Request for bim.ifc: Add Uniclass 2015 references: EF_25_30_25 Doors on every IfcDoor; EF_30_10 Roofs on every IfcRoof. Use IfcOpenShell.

First a look at what the model holds.

```python
import ifcopenshell

model = ifcopenshell.open("bim.ifc")
print(model.schema)
print("classifications:", [c.Name for c in model.by_type("IfcClassification")])
for ifc_class in ("IfcDoor", "IfcRoof", "IfcStair", "IfcWall", "IfcWindow"):
    print(ifc_class, len(model.by_type(ifc_class)))
```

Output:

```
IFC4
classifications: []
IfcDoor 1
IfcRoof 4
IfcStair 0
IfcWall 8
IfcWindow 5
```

```python
import ifcopenshell
import ifcopenshell.api.classification

model = ifcopenshell.open("bim.ifc")

system = ifcopenshell.api.classification.add_classification(model, classification="Uniclass 2015")

codes = {
    "IfcDoor": ("EF_25_30_25", "Doors"),
    "IfcRoof": ("EF_30_10", "Roofs"),
}
for ifc_class, (code, name) in codes.items():
    products = model.by_type(ifc_class)
    ifcopenshell.api.classification.add_reference(
        model, products=products, classification=system, identification=code, name=name
    )
    print(code, len(products))

model.write("bim_rev.ifc")
```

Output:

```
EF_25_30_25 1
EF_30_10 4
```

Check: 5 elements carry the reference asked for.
